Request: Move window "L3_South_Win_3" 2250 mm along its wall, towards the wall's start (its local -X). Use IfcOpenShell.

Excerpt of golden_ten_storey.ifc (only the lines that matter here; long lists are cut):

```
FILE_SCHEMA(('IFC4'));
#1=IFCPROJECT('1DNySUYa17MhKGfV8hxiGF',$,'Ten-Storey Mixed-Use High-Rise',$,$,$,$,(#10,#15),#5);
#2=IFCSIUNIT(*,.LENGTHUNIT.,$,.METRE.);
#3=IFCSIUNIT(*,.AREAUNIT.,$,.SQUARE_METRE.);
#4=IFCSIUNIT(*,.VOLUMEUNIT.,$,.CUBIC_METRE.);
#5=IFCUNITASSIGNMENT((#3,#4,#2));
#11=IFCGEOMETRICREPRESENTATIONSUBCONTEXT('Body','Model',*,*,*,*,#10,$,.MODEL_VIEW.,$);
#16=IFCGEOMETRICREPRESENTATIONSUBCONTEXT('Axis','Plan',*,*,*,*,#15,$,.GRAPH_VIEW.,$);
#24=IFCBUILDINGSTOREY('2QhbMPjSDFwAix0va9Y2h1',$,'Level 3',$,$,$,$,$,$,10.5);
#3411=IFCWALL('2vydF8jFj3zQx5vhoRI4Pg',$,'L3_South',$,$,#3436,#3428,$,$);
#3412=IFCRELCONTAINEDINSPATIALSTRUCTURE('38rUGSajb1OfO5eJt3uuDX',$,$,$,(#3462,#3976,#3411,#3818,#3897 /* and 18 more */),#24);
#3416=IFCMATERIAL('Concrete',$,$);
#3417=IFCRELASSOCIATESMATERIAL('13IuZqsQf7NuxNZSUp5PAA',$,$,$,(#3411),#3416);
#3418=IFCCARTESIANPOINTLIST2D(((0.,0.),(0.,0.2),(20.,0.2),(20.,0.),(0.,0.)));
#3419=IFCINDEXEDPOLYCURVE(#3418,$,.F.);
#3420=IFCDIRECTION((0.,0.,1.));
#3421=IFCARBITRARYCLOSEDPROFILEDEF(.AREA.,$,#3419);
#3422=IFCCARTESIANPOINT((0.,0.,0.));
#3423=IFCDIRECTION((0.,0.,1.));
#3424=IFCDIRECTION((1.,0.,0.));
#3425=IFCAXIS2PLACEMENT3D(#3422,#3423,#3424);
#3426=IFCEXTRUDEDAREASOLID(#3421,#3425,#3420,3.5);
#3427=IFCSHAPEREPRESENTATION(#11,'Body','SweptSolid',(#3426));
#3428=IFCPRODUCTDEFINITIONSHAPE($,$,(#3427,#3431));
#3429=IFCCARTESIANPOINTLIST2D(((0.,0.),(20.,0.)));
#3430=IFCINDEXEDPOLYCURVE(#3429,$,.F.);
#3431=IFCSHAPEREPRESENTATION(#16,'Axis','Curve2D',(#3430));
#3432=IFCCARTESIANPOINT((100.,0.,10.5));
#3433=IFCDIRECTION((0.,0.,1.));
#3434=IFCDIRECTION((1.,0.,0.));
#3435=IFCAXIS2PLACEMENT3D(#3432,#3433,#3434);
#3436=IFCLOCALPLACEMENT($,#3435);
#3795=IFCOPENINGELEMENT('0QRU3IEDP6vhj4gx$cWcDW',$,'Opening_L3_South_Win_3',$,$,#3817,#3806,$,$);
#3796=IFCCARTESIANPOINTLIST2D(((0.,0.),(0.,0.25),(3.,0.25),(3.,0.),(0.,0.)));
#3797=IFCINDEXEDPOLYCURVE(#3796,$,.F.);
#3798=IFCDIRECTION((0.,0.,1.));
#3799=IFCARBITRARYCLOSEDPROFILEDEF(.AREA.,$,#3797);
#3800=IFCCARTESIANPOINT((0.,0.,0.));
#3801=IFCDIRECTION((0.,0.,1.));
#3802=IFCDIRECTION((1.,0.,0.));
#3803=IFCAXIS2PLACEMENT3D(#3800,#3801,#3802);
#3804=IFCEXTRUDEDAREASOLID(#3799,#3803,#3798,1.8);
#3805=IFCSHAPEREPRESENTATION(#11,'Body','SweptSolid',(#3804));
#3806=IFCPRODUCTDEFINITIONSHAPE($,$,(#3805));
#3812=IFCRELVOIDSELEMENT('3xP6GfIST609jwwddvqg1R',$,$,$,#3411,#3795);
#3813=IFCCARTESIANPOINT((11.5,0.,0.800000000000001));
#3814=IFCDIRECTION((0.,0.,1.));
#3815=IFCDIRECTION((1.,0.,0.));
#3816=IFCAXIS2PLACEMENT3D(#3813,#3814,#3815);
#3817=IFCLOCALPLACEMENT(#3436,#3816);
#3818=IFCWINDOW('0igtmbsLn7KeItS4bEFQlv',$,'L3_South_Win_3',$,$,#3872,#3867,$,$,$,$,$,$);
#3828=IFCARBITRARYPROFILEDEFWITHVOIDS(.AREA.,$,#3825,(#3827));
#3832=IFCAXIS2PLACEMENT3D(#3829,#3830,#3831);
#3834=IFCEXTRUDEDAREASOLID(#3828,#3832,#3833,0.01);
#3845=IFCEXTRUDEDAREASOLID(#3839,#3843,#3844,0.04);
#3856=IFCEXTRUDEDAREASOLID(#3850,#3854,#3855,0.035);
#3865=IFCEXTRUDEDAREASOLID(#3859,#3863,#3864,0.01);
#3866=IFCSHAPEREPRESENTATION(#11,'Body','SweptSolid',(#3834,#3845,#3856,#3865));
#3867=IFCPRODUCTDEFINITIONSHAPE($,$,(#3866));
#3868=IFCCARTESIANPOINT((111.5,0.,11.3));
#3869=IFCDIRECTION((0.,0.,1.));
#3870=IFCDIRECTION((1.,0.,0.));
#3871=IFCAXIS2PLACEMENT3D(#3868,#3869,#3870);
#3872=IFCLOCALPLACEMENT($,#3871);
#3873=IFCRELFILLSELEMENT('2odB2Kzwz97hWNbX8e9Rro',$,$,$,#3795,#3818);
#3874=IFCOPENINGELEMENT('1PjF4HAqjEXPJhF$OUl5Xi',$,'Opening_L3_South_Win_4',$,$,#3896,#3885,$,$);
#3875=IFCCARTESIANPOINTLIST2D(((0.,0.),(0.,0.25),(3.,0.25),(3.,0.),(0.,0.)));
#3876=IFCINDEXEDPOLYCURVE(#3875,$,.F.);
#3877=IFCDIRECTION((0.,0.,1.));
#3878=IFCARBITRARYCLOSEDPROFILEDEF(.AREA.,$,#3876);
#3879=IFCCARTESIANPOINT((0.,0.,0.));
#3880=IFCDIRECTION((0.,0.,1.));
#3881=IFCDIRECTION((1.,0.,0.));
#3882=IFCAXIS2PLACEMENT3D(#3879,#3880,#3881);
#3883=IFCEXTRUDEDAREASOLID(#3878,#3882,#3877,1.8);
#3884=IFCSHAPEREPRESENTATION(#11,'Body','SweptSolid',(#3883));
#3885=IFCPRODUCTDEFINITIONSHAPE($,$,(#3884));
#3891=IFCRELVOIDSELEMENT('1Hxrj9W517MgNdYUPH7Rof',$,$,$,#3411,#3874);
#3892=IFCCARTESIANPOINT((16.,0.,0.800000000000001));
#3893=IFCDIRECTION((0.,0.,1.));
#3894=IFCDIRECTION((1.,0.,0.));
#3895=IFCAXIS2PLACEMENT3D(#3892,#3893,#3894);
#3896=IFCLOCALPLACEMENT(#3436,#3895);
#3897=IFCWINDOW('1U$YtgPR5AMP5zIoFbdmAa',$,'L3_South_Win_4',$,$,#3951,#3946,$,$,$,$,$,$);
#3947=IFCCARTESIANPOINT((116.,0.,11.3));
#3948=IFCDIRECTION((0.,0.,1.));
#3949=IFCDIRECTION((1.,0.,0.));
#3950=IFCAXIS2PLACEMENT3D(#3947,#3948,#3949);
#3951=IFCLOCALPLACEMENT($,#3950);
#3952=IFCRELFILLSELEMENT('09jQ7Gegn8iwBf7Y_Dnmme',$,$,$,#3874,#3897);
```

```python
import ifcopenshell
import ifcopenshell.api.geometry
import ifcopenshell.util.placement
import ifcopenshell.util.unit

model = ifcopenshell.open("golden_ten_storey.ifc")
unit_scale = ifcopenshell.util.unit.calculate_unit_scale(model)

window = model.by_guid("0igtmbsLn7KeItS4bEFQlv")
opening = window.FillsVoids[0].RelatingOpeningElement
wall = opening.VoidsElements[0].RelatingBuildingElement

wall_matrix = ifcopenshell.util.placement.get_local_placement(wall.ObjectPlacement)
shift = wall_matrix[:3, 0] * -2.25 / unit_scale
before = ifcopenshell.util.placement.get_local_placement(window.ObjectPlacement)[:3, 3].copy()

# The window is not placed relative to its opening, so move both.
for product in (opening, window):
    matrix = ifcopenshell.util.placement.get_local_placement(product.ObjectPlacement)
    matrix[:3, 3] += shift
    ifcopenshell.api.geometry.edit_object_placement(model, product=product, matrix=matrix, is_si=False)

after = ifcopenshell.util.placement.get_local_placement(window.ObjectPlacement)[:3, 3]
print("window moved by", (after - before).round(3) + 0.0)

model.write("golden_ten_storey-out.ifc")
```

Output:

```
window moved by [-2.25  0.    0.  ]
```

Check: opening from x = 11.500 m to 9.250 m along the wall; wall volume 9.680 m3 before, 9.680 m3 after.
